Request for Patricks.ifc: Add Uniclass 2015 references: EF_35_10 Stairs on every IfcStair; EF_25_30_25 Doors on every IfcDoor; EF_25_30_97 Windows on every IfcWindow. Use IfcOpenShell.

First a look at what the model holds.

```python
import ifcopenshell

model = ifcopenshell.open("Patricks.ifc")
print(model.schema)
print("classifications:", [c.Name for c in model.by_type("IfcClassification")])
for ifc_class in ("IfcDoor", "IfcRoof", "IfcStair", "IfcWall", "IfcWindow"):
    print(ifc_class, len(model.by_type(ifc_class)))
```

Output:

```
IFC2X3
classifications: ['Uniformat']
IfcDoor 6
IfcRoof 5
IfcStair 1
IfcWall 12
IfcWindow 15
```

```python
import ifcopenshell
import ifcopenshell.api.classification

model = ifcopenshell.open("Patricks.ifc")

# IFC2X3 requires Source and Edition and has no link from the project to the system.
system = model.create_entity("IfcClassification", Source="NBS", Edition="2015", Name="Uniclass 2015")

codes = {
    "IfcStair": ("EF_35_10", "Stairs"),
    "IfcDoor": ("EF_25_30_25", "Doors"),
    "IfcWindow": ("EF_25_30_97", "Windows"),
}
for ifc_class, (code, name) in codes.items():
    products = model.by_type(ifc_class)
    ifcopenshell.api.classification.add_reference(
        model, products=products, classification=system, identification=code, name=name
    )
    print(code, len(products))

model.write("Patricks-out.ifc")
```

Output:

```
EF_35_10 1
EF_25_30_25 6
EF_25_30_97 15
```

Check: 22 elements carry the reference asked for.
